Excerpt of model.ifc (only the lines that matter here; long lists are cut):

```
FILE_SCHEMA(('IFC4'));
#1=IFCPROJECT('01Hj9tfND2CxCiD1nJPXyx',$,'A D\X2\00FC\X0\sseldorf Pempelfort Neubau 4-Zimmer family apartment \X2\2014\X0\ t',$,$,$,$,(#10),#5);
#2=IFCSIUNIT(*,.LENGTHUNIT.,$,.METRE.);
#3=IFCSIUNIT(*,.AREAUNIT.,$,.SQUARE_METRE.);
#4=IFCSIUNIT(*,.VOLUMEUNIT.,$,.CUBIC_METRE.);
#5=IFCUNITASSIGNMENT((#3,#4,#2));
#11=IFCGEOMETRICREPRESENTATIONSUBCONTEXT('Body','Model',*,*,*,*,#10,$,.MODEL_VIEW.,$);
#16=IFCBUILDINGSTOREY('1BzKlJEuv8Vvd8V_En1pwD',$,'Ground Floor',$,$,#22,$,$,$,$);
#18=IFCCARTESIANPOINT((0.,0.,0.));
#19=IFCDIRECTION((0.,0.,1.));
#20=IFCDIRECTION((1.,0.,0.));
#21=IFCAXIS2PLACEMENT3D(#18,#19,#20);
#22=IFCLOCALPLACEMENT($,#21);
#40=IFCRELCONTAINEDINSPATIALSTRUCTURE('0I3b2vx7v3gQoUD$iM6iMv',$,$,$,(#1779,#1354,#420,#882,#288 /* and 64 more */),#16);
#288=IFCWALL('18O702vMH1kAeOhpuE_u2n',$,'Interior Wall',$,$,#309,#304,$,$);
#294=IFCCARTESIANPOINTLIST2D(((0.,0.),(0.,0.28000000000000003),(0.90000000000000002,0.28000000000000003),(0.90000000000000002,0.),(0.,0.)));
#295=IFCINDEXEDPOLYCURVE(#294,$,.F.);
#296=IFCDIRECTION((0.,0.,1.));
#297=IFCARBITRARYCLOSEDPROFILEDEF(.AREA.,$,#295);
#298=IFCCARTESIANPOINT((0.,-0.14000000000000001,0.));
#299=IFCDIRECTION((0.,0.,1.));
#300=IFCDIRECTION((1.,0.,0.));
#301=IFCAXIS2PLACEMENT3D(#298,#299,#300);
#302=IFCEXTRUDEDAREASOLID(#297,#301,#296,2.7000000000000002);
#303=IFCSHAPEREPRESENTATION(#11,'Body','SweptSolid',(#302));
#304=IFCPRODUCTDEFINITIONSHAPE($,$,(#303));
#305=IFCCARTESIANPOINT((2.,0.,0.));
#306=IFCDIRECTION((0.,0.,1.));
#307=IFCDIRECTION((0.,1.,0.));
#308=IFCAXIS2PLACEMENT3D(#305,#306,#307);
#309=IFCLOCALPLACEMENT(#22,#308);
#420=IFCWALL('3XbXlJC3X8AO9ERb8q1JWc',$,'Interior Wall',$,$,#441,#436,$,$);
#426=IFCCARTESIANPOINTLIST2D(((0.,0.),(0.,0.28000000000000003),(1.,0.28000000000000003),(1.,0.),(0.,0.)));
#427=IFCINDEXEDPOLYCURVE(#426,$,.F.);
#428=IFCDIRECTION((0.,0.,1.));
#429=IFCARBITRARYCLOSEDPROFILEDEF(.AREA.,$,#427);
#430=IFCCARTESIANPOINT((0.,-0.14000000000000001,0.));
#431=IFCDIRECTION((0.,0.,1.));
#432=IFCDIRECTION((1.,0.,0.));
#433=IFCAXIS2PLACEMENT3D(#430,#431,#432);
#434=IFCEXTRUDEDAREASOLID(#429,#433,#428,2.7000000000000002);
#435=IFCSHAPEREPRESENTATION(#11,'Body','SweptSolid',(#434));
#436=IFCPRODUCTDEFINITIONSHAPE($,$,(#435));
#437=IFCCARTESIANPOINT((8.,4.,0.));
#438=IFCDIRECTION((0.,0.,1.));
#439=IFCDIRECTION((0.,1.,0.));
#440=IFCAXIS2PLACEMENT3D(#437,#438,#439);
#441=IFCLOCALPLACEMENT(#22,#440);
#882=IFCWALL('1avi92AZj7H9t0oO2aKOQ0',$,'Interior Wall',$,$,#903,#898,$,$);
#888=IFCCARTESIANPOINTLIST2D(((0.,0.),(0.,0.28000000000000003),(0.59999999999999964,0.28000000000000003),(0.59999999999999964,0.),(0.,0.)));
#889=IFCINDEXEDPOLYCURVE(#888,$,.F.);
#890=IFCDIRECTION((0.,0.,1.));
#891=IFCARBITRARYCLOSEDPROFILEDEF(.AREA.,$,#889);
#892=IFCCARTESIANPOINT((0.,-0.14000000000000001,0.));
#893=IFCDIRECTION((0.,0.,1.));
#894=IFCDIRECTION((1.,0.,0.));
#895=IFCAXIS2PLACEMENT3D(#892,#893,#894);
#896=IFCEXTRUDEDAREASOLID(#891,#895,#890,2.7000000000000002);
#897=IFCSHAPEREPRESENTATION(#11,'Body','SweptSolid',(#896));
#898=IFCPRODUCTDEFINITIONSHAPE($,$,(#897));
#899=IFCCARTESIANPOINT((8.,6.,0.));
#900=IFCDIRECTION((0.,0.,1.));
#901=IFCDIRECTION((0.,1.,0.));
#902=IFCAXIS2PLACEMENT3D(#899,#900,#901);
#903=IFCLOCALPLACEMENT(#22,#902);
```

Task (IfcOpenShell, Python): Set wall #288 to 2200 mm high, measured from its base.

```python
import ifcopenshell
import ifcopenshell.geom
import ifcopenshell.util.representation
import ifcopenshell.util.shape

model = ifcopenshell.open("model.ifc")
settings = ifcopenshell.geom.settings()


def volume(element):
    """Net volume in cubic metres, openings subtracted."""
    shape = ifcopenshell.geom.create_shape(settings, element)
    return ifcopenshell.util.shape.get_volume(shape.geometry)


wall = model.by_id(288)
before = volume(wall)

body = ifcopenshell.util.representation.get_representation(wall, "Model", "Body")
solid = body.Items[0]
old_height = solid.Depth
solid.Depth = 2.2
after = volume(wall)

print(f"height {old_height:g} -> {solid.Depth:g}, volume {before:.3f} -> {after:.3f} m3")

model.write("model_updated.ifc")
```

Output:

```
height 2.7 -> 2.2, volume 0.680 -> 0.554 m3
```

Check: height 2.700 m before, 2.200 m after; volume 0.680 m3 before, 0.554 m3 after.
